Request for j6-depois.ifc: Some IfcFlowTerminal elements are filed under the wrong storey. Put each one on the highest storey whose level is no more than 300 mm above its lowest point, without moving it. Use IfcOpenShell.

First a look at what the model holds.

```python
import ifcopenshell
import ifcopenshell.util.element
import ifcopenshell.util.placement

model = ifcopenshell.open("j6-depois.ifc")
print(model.schema)
for storey in model.by_type("IfcBuildingStorey"):
    level = ifcopenshell.util.placement.get_storey_elevation(storey)
    count = sum(e.is_a("IfcFlowTerminal") for e in ifcopenshell.util.element.get_contained(storey))
    print(storey.id(), storey.Name, round(level, 3), count, sep=" | ")
```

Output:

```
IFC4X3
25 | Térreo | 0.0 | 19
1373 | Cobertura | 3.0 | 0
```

```python
import ifcopenshell
import ifcopenshell.api.spatial
import ifcopenshell.geom
import ifcopenshell.util.element
import ifcopenshell.util.placement
import ifcopenshell.util.shape
import ifcopenshell.util.unit

model = ifcopenshell.open("j6-depois.ifc")
unit_scale = ifcopenshell.util.unit.calculate_unit_scale(model)
settings = ifcopenshell.geom.settings()

levels = sorted(
    ((ifcopenshell.util.placement.get_storey_elevation(s) * unit_scale, s) for s in model.by_type("IfcBuildingStorey")),
    key=lambda pair: pair[0],
)

for e in model.by_type("IfcFlowTerminal"):
    current = e.ContainedInStructure[0].RelatingStructure if e.ContainedInStructure else None
    if current is None or not current.is_a("IfcBuildingStorey"):
        continue
    shape = ifcopenshell.geom.create_shape(settings, e)
    bottom = ifcopenshell.util.shape.get_shape_bottom_elevation(shape, shape.geometry)
    below = [s for level, s in levels if level <= bottom + 0.3]
    storey = below[-1] if below else levels[0][1]
    if storey != current:
        # assign_container keeps the world position.
        ifcopenshell.api.spatial.assign_container(model, products=[e], relating_structure=storey)
        print(e.id(), current.Name, "->", storey.Name)

model.write("j6-depois_v2.ifc")
```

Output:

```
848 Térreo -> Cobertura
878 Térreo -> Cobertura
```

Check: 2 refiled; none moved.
